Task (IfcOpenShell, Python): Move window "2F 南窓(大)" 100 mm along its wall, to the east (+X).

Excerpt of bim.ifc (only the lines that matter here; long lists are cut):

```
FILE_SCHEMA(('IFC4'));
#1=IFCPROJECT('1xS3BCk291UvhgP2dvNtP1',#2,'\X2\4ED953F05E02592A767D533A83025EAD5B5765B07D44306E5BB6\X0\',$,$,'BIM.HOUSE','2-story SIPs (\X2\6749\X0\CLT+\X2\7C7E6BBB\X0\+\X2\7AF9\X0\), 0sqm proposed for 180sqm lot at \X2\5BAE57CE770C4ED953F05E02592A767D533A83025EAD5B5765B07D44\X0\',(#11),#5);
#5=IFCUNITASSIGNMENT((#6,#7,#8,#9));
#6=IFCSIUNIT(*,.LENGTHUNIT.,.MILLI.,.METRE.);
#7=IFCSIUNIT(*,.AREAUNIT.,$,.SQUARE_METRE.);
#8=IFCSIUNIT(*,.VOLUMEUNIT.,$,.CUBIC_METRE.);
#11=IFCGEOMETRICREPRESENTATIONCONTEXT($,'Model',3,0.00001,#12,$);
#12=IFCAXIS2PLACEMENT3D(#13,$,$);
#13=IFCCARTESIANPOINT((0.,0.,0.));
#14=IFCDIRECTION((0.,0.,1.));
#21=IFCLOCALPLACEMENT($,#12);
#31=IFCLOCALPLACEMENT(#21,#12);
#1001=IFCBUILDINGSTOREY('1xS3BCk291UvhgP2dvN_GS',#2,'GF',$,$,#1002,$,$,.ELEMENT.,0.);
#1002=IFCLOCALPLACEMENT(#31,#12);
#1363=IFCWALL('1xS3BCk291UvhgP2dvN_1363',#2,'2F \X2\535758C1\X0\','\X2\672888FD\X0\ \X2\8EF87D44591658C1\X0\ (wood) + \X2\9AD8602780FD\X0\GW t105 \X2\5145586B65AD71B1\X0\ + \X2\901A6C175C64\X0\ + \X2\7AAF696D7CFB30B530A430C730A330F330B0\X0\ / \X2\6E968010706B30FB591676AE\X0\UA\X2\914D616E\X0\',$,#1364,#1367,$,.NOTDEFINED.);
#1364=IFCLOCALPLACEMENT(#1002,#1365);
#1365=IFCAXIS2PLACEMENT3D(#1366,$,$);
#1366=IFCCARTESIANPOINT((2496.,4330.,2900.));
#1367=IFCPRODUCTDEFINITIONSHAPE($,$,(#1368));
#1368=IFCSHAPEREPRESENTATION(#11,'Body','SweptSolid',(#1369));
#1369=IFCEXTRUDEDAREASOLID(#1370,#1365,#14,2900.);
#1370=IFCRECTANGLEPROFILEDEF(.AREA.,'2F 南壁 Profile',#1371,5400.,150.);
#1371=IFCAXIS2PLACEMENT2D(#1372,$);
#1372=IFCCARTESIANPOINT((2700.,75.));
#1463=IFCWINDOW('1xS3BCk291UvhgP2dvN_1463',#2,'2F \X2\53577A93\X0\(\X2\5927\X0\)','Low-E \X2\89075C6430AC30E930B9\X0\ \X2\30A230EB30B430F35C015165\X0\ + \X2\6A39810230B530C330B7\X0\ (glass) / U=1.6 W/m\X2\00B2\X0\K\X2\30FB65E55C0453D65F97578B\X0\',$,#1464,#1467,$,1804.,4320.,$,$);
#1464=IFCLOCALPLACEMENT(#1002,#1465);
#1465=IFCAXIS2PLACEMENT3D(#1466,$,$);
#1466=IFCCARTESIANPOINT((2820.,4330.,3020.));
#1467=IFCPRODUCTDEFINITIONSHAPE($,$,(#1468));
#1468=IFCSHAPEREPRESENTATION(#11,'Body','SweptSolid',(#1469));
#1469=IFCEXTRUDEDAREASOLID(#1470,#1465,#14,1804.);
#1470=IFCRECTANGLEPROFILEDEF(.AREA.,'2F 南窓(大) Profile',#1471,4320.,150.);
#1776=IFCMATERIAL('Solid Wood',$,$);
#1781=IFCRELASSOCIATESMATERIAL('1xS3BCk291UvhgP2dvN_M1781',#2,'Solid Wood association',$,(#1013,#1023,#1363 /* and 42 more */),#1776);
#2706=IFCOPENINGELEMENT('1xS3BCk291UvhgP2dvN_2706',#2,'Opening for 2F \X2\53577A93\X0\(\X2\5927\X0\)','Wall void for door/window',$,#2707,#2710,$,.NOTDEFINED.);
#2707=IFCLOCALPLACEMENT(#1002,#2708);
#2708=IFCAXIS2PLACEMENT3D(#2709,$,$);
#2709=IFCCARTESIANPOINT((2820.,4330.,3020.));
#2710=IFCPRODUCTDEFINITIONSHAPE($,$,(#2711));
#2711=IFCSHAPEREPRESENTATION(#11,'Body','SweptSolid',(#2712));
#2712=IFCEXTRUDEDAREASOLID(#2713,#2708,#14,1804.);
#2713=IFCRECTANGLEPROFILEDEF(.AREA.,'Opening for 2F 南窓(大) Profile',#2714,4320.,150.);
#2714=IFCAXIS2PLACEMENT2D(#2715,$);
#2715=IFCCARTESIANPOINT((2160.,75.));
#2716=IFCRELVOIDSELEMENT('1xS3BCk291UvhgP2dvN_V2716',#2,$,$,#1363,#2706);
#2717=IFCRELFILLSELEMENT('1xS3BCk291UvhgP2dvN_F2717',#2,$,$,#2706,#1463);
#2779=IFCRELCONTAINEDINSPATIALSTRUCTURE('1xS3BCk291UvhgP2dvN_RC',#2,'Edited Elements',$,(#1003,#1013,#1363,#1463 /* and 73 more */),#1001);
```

```python
import ifcopenshell
import ifcopenshell.api.geometry
import ifcopenshell.util.placement
import ifcopenshell.util.unit

model = ifcopenshell.open("bim.ifc")
unit_scale = ifcopenshell.util.unit.calculate_unit_scale(model)

window = model.by_guid("1xS3BCk291UvhgP2dvN_1463")
opening = window.FillsVoids[0].RelatingOpeningElement
wall = opening.VoidsElements[0].RelatingBuildingElement

wall_matrix = ifcopenshell.util.placement.get_local_placement(wall.ObjectPlacement)
shift = wall_matrix[:3, 0] * 0.1 / unit_scale
before = ifcopenshell.util.placement.get_local_placement(window.ObjectPlacement)[:3, 3].copy()

# The window is not placed relative to its opening, so move both.
for product in (opening, window):
    matrix = ifcopenshell.util.placement.get_local_placement(product.ObjectPlacement)
    matrix[:3, 3] += shift
    ifcopenshell.api.geometry.edit_object_placement(model, product=product, matrix=matrix, is_si=False)

after = ifcopenshell.util.placement.get_local_placement(window.ObjectPlacement)[:3, 3]
print("window moved by", (after - before).round(3) + 0.0)

model.write("bim_edited.ifc")
```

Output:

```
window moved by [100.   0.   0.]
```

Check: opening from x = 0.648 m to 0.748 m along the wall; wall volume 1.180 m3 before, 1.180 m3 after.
